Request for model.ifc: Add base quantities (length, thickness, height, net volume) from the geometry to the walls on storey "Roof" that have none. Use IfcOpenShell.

First a look at what the model holds.

```python
import ifcopenshell
import ifcopenshell.util.element
import ifcopenshell.util.unit

model = ifcopenshell.open("model.ifc")
print(model.schema)
for unit_type in ("LENGTHUNIT", "AREAUNIT", "VOLUMEUNIT"):
    print(unit_type, ifcopenshell.util.unit.calculate_unit_scale(model, unit_type))
storey = next(s for s in model.by_type("IfcBuildingStorey") if s.Name == "Roof")
walls = [e for e in ifcopenshell.util.element.get_decomposition(storey) if e.is_a("IfcWall")]
for e in sorted(walls, key=lambda e: e.id()):
    print(e.id(), e.is_a(), e.Name, list(ifcopenshell.util.element.get_psets(e, qtos_only=True)), sep=" | ")
```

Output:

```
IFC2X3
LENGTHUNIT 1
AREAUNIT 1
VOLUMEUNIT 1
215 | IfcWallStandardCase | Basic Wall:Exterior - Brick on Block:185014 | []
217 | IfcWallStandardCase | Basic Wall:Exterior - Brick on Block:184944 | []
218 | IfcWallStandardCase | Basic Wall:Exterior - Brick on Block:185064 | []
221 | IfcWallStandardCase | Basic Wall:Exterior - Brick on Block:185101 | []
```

```python
import ifcopenshell
import ifcopenshell.api.pset
import ifcopenshell.geom
import ifcopenshell.util.element
import ifcopenshell.util.shape
import ifcopenshell.util.unit

model = ifcopenshell.open("model.ifc")
unit_scale = ifcopenshell.util.unit.calculate_unit_scale(model)
volume_scale = ifcopenshell.util.unit.calculate_unit_scale(model, "VOLUMEUNIT")
settings = ifcopenshell.geom.settings()

storey = next(s for s in model.by_type("IfcBuildingStorey") if s.Name == "Roof")
walls = [e for e in ifcopenshell.util.element.get_decomposition(storey) if e.is_a("IfcWall")]

for e in sorted(walls, key=lambda e: e.id()):
    if ifcopenshell.util.element.get_psets(e, qtos_only=True, should_inherit=False):
        continue
    # Geometry comes back in metres, in the element's own axes.
    shape = ifcopenshell.geom.create_shape(settings, e)
    values = {
        "Length": ifcopenshell.util.shape.get_x(shape.geometry) / unit_scale,
        "Width": ifcopenshell.util.shape.get_y(shape.geometry) / unit_scale,
        "Height": ifcopenshell.util.shape.get_z(shape.geometry) / unit_scale,
        "NetVolume": ifcopenshell.util.shape.get_volume(shape.geometry) / volume_scale,
    }
    qto = ifcopenshell.api.pset.add_qto(model, product=e, name="BaseQuantities")
    ifcopenshell.api.pset.edit_qto(model, qto=qto, properties=values)
    print(e.id(), {k: round(v, 3) for k, v in values.items()})

model.write("model_edited.ifc")
```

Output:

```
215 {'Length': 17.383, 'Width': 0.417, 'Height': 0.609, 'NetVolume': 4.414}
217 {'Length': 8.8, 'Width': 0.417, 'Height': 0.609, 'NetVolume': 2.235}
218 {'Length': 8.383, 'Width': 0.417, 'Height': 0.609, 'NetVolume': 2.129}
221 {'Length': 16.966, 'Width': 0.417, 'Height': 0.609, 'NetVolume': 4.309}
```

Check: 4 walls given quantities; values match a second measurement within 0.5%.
